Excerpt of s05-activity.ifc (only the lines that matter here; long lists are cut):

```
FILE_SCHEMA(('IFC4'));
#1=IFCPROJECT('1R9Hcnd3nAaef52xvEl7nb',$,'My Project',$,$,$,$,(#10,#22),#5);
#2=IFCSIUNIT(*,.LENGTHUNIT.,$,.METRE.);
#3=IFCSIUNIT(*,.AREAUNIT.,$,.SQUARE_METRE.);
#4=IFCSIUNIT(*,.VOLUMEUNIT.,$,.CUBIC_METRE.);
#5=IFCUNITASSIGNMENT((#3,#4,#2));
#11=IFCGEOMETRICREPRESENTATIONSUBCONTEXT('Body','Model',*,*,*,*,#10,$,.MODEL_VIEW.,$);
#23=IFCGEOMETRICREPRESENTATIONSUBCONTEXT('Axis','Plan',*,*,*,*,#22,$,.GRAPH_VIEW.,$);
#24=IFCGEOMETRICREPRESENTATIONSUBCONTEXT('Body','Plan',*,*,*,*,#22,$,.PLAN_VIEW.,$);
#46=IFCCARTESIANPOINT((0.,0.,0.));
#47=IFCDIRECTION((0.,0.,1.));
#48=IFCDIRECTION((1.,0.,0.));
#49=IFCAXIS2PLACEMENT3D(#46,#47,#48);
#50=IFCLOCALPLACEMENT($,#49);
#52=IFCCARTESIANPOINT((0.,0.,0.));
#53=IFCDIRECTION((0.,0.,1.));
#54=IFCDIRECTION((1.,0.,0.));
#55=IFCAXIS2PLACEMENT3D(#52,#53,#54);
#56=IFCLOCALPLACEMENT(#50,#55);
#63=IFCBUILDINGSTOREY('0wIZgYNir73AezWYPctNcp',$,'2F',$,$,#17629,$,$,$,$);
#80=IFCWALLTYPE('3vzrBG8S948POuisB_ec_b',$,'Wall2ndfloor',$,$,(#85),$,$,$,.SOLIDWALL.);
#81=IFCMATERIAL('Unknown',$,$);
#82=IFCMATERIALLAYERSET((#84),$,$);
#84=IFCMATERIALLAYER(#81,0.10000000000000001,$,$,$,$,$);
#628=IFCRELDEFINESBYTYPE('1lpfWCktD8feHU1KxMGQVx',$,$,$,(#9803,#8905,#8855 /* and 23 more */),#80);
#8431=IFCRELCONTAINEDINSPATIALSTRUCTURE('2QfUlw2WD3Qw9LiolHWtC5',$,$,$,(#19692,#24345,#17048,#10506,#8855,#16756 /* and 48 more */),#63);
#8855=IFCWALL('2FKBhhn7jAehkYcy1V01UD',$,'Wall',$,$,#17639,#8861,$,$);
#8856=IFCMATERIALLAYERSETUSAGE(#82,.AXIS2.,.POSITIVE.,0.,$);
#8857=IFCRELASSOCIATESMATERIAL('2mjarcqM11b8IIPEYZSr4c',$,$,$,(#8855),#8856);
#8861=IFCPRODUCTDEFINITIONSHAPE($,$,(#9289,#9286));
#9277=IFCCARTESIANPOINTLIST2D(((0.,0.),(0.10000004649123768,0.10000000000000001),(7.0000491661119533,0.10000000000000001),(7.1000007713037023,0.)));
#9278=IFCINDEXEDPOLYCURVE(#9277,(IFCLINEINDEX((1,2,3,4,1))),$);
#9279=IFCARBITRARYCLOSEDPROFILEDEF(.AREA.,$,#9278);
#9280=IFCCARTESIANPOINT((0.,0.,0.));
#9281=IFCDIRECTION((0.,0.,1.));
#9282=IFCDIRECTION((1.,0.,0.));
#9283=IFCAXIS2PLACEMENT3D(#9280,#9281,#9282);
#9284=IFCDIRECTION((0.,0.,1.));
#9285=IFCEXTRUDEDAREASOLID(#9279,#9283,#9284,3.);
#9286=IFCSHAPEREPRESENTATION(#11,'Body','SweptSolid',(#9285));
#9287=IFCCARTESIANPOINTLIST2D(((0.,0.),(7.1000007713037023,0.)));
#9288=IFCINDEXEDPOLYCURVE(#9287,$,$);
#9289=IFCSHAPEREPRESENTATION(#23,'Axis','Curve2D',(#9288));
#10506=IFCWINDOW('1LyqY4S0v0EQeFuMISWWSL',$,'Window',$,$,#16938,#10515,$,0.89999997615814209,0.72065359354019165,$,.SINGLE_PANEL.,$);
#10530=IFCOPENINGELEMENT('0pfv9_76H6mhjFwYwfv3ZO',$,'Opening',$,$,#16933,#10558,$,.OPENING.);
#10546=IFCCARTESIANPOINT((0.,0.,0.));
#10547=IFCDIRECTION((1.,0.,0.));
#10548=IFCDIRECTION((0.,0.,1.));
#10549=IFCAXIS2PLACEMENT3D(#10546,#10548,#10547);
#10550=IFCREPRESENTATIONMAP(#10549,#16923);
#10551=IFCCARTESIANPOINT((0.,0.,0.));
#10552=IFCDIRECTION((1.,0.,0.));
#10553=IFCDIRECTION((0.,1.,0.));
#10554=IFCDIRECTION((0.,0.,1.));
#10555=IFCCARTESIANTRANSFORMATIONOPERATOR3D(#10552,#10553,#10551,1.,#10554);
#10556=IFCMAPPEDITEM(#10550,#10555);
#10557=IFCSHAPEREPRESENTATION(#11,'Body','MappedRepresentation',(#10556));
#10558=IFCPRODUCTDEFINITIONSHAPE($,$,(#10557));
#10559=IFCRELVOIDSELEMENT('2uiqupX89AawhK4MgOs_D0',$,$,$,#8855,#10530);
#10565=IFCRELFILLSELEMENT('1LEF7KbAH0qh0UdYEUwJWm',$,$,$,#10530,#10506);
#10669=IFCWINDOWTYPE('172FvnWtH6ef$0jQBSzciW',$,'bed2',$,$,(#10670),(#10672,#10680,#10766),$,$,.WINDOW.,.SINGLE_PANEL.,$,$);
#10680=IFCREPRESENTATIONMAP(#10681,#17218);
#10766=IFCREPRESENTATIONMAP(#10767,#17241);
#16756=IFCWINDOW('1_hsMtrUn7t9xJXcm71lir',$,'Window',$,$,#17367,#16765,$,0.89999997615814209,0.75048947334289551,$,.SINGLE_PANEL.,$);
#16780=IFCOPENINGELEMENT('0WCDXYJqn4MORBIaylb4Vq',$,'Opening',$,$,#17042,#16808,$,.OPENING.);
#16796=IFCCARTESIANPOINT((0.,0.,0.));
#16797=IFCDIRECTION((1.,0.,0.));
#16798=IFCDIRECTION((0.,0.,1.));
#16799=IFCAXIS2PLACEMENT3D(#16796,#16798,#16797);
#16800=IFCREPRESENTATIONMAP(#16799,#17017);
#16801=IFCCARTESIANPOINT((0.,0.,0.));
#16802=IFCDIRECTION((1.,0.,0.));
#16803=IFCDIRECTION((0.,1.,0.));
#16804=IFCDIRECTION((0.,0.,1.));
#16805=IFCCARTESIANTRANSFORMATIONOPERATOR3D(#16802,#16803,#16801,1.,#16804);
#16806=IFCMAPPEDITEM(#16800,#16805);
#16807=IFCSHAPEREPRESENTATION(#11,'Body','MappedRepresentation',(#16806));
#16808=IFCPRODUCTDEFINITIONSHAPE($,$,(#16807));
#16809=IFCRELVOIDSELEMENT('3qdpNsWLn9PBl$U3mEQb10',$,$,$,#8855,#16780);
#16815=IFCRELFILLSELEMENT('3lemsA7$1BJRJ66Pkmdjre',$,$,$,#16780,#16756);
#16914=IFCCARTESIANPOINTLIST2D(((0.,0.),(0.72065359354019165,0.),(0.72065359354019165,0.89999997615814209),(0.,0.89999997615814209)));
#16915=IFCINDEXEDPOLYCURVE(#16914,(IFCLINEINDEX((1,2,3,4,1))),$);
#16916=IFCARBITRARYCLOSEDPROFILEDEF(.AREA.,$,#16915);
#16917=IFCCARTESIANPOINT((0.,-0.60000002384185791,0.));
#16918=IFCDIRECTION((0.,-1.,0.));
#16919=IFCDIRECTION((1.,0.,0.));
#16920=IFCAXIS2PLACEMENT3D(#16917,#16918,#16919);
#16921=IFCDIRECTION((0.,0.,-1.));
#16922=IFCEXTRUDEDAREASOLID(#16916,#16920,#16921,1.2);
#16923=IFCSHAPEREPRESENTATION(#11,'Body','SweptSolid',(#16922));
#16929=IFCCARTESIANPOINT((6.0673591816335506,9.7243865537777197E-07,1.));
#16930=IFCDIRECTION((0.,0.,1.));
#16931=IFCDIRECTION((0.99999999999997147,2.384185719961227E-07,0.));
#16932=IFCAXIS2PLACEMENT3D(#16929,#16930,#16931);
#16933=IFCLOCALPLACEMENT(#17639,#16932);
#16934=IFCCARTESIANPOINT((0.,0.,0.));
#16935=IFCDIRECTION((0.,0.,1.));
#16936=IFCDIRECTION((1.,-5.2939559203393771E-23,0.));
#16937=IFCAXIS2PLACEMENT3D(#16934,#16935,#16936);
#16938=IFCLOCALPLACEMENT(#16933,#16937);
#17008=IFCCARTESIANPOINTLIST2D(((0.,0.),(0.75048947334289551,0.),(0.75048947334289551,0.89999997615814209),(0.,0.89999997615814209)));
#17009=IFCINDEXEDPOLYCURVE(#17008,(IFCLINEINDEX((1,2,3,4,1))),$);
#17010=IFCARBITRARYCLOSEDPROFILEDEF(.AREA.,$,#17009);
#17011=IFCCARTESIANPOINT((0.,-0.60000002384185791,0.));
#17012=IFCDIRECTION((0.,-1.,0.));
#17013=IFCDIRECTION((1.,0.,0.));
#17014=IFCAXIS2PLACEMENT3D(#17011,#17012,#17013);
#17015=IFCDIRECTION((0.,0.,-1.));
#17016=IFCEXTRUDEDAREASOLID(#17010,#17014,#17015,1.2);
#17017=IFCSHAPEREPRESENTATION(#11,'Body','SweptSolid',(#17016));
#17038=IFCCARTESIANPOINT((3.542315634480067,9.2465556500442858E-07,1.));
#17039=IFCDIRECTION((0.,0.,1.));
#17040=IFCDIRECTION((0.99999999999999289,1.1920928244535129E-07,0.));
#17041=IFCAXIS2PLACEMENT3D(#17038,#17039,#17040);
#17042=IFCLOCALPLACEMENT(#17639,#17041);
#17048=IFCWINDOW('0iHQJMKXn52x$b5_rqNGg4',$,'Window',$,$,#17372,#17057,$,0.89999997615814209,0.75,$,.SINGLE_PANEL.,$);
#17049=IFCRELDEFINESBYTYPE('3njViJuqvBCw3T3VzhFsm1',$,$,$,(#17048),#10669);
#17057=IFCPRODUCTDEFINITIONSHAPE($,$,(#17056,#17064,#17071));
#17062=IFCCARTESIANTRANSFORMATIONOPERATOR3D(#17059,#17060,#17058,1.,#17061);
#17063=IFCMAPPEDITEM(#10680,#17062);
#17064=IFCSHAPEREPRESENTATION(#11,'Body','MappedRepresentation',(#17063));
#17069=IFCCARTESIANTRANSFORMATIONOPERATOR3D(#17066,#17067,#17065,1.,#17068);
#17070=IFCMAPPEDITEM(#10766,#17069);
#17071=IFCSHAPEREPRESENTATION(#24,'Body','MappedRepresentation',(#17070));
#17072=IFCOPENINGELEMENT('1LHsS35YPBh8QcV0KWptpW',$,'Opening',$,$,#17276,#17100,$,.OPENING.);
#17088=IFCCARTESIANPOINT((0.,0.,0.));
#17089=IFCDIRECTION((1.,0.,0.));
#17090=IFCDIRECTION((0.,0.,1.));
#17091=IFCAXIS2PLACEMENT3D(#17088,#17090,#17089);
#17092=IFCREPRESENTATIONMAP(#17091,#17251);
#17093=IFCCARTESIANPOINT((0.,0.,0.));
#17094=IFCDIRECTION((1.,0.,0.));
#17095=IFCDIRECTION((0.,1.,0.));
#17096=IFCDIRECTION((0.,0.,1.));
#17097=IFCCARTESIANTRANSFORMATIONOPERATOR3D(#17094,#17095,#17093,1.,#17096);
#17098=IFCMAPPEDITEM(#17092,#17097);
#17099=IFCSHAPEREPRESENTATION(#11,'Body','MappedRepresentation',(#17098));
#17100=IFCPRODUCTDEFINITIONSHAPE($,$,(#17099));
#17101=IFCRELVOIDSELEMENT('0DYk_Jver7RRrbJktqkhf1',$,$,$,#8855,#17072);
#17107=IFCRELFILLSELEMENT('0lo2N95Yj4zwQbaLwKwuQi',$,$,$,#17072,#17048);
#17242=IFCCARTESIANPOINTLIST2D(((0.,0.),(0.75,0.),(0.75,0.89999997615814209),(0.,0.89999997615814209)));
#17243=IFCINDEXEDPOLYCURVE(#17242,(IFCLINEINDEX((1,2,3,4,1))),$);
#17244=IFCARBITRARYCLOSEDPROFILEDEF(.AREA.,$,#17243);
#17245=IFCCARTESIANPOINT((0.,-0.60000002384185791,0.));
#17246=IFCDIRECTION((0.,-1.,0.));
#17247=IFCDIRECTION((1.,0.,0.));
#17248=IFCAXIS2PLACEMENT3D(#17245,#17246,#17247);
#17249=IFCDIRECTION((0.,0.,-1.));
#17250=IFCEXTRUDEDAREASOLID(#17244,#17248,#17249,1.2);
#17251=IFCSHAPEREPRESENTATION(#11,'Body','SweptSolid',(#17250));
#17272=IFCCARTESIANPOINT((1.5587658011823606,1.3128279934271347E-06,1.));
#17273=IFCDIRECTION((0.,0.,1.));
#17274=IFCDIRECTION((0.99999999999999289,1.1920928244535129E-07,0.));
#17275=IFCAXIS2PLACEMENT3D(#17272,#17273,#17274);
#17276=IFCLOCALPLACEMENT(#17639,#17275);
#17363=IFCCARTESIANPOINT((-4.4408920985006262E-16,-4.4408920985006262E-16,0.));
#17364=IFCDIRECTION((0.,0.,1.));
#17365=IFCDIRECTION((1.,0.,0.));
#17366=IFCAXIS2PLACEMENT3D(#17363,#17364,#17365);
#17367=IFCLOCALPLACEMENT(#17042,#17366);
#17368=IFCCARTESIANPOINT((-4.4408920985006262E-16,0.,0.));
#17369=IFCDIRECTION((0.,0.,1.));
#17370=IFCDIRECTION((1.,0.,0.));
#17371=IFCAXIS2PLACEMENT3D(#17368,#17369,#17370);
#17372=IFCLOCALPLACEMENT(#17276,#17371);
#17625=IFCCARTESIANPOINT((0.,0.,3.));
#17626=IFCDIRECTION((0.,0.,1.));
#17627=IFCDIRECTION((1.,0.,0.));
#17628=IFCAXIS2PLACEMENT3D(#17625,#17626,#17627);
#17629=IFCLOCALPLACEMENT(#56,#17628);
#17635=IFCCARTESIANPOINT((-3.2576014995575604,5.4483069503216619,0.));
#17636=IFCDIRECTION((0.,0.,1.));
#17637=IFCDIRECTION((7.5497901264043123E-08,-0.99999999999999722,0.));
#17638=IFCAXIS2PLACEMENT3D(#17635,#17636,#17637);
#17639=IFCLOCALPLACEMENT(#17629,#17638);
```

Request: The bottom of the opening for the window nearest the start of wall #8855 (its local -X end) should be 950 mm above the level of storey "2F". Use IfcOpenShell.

```python
import numpy as np
import ifcopenshell
import ifcopenshell.api.geometry
import ifcopenshell.geom
import ifcopenshell.util.element
import ifcopenshell.util.placement
import ifcopenshell.util.shape
import ifcopenshell.util.unit

model = ifcopenshell.open("s05-activity.ifc")
unit_scale = ifcopenshell.util.unit.calculate_unit_scale(model)

window = model.by_guid("0iHQJMKXn52x$b5_rqNGg4")
opening = window.FillsVoids[0].RelatingOpeningElement
storey = ifcopenshell.util.element.get_container(window, ifc_class="IfcBuildingStorey")
level = ifcopenshell.util.placement.get_local_placement(storey.ObjectPlacement)[2, 3]

# The opening's origin need not be at the sill, so measure its lowest point.
shape = ifcopenshell.geom.create_shape(ifcopenshell.geom.settings(), opening)
bottom = ifcopenshell.util.shape.get_shape_bottom_elevation(shape, shape.geometry) / unit_scale
dz = level + 0.95 / unit_scale - bottom

shift = np.array([0.0, 0.0, dz])
# The window is placed relative to its opening, so it follows when the opening moves.
matrix = ifcopenshell.util.placement.get_local_placement(opening.ObjectPlacement)
matrix[:3, 3] += shift
ifcopenshell.api.geometry.edit_object_placement(
    model, product=opening, matrix=matrix, is_si=False, should_transform_children=True
)

print(f"moved by {dz * unit_scale:+.3f} m")

model.write("s05-activity_rev.ifc")
```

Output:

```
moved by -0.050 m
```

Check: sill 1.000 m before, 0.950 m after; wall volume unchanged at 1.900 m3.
